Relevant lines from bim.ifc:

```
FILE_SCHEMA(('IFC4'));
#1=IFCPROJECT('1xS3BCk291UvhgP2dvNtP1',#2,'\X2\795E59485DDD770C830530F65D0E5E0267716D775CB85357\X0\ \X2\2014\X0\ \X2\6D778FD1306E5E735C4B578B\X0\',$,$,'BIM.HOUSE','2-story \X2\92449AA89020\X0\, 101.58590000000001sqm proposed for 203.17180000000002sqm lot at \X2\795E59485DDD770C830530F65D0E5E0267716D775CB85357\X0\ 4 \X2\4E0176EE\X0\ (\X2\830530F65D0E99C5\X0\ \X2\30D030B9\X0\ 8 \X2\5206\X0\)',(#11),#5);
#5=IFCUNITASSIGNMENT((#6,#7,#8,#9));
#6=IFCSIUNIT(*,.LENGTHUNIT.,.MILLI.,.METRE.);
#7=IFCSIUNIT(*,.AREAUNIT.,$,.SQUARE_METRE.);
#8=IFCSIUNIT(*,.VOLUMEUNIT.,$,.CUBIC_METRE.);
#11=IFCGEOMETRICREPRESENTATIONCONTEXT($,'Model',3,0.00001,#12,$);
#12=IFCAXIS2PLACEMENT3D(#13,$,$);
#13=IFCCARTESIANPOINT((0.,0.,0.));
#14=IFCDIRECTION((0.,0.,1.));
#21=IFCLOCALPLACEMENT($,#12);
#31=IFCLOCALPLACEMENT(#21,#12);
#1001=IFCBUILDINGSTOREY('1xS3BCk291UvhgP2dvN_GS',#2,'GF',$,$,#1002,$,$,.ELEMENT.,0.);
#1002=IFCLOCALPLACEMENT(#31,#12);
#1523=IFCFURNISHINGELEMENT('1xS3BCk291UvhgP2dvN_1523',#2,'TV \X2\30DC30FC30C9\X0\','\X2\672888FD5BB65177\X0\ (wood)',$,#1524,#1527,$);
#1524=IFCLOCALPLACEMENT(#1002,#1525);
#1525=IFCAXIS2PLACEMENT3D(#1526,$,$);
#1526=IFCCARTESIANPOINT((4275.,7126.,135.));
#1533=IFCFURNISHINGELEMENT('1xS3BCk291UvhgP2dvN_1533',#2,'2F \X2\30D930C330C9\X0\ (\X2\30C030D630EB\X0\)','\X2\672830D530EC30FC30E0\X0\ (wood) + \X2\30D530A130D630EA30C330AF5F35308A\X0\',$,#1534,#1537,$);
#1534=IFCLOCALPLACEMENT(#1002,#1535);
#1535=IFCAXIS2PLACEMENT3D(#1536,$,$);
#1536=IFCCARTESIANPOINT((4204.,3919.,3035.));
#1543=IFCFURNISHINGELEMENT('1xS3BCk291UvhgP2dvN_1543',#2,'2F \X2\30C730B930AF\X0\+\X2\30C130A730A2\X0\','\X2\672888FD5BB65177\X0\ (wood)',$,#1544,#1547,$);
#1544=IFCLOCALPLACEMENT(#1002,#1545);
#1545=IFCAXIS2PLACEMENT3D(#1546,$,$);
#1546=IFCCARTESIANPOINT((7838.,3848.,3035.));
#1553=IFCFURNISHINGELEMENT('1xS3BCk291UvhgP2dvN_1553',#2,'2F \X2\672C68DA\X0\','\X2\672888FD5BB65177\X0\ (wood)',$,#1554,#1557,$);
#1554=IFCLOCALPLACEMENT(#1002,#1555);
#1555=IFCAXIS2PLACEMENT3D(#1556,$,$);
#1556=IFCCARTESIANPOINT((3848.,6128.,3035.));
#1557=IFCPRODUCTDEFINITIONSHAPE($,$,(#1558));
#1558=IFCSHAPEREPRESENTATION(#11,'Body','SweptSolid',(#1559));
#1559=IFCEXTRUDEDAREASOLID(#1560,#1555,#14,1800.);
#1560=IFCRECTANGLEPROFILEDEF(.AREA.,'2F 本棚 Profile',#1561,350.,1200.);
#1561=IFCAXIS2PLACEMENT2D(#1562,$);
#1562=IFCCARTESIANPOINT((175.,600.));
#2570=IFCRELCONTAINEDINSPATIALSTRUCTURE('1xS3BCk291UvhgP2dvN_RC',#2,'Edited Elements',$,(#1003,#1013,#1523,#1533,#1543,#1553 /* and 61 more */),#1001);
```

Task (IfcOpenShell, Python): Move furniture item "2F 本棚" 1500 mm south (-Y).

```python
import ifcopenshell
import ifcopenshell.api.geometry
import ifcopenshell.util.placement

model = ifcopenshell.open("bim.ifc")

item = model.by_guid("1xS3BCk291UvhgP2dvN_1553")
matrix = ifcopenshell.util.placement.get_local_placement(item.ObjectPlacement)
matrix[1, 3] -= 1500.0
ifcopenshell.api.geometry.edit_object_placement(model, product=item, matrix=matrix, is_si=False)

print(ifcopenshell.util.placement.get_local_placement(item.ObjectPlacement).round(3) + 0.0)

model.write("bim_updated.ifc")
```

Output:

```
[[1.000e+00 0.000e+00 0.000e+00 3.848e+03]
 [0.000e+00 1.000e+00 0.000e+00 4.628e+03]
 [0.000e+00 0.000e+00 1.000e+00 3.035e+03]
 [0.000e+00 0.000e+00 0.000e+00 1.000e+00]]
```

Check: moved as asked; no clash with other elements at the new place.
